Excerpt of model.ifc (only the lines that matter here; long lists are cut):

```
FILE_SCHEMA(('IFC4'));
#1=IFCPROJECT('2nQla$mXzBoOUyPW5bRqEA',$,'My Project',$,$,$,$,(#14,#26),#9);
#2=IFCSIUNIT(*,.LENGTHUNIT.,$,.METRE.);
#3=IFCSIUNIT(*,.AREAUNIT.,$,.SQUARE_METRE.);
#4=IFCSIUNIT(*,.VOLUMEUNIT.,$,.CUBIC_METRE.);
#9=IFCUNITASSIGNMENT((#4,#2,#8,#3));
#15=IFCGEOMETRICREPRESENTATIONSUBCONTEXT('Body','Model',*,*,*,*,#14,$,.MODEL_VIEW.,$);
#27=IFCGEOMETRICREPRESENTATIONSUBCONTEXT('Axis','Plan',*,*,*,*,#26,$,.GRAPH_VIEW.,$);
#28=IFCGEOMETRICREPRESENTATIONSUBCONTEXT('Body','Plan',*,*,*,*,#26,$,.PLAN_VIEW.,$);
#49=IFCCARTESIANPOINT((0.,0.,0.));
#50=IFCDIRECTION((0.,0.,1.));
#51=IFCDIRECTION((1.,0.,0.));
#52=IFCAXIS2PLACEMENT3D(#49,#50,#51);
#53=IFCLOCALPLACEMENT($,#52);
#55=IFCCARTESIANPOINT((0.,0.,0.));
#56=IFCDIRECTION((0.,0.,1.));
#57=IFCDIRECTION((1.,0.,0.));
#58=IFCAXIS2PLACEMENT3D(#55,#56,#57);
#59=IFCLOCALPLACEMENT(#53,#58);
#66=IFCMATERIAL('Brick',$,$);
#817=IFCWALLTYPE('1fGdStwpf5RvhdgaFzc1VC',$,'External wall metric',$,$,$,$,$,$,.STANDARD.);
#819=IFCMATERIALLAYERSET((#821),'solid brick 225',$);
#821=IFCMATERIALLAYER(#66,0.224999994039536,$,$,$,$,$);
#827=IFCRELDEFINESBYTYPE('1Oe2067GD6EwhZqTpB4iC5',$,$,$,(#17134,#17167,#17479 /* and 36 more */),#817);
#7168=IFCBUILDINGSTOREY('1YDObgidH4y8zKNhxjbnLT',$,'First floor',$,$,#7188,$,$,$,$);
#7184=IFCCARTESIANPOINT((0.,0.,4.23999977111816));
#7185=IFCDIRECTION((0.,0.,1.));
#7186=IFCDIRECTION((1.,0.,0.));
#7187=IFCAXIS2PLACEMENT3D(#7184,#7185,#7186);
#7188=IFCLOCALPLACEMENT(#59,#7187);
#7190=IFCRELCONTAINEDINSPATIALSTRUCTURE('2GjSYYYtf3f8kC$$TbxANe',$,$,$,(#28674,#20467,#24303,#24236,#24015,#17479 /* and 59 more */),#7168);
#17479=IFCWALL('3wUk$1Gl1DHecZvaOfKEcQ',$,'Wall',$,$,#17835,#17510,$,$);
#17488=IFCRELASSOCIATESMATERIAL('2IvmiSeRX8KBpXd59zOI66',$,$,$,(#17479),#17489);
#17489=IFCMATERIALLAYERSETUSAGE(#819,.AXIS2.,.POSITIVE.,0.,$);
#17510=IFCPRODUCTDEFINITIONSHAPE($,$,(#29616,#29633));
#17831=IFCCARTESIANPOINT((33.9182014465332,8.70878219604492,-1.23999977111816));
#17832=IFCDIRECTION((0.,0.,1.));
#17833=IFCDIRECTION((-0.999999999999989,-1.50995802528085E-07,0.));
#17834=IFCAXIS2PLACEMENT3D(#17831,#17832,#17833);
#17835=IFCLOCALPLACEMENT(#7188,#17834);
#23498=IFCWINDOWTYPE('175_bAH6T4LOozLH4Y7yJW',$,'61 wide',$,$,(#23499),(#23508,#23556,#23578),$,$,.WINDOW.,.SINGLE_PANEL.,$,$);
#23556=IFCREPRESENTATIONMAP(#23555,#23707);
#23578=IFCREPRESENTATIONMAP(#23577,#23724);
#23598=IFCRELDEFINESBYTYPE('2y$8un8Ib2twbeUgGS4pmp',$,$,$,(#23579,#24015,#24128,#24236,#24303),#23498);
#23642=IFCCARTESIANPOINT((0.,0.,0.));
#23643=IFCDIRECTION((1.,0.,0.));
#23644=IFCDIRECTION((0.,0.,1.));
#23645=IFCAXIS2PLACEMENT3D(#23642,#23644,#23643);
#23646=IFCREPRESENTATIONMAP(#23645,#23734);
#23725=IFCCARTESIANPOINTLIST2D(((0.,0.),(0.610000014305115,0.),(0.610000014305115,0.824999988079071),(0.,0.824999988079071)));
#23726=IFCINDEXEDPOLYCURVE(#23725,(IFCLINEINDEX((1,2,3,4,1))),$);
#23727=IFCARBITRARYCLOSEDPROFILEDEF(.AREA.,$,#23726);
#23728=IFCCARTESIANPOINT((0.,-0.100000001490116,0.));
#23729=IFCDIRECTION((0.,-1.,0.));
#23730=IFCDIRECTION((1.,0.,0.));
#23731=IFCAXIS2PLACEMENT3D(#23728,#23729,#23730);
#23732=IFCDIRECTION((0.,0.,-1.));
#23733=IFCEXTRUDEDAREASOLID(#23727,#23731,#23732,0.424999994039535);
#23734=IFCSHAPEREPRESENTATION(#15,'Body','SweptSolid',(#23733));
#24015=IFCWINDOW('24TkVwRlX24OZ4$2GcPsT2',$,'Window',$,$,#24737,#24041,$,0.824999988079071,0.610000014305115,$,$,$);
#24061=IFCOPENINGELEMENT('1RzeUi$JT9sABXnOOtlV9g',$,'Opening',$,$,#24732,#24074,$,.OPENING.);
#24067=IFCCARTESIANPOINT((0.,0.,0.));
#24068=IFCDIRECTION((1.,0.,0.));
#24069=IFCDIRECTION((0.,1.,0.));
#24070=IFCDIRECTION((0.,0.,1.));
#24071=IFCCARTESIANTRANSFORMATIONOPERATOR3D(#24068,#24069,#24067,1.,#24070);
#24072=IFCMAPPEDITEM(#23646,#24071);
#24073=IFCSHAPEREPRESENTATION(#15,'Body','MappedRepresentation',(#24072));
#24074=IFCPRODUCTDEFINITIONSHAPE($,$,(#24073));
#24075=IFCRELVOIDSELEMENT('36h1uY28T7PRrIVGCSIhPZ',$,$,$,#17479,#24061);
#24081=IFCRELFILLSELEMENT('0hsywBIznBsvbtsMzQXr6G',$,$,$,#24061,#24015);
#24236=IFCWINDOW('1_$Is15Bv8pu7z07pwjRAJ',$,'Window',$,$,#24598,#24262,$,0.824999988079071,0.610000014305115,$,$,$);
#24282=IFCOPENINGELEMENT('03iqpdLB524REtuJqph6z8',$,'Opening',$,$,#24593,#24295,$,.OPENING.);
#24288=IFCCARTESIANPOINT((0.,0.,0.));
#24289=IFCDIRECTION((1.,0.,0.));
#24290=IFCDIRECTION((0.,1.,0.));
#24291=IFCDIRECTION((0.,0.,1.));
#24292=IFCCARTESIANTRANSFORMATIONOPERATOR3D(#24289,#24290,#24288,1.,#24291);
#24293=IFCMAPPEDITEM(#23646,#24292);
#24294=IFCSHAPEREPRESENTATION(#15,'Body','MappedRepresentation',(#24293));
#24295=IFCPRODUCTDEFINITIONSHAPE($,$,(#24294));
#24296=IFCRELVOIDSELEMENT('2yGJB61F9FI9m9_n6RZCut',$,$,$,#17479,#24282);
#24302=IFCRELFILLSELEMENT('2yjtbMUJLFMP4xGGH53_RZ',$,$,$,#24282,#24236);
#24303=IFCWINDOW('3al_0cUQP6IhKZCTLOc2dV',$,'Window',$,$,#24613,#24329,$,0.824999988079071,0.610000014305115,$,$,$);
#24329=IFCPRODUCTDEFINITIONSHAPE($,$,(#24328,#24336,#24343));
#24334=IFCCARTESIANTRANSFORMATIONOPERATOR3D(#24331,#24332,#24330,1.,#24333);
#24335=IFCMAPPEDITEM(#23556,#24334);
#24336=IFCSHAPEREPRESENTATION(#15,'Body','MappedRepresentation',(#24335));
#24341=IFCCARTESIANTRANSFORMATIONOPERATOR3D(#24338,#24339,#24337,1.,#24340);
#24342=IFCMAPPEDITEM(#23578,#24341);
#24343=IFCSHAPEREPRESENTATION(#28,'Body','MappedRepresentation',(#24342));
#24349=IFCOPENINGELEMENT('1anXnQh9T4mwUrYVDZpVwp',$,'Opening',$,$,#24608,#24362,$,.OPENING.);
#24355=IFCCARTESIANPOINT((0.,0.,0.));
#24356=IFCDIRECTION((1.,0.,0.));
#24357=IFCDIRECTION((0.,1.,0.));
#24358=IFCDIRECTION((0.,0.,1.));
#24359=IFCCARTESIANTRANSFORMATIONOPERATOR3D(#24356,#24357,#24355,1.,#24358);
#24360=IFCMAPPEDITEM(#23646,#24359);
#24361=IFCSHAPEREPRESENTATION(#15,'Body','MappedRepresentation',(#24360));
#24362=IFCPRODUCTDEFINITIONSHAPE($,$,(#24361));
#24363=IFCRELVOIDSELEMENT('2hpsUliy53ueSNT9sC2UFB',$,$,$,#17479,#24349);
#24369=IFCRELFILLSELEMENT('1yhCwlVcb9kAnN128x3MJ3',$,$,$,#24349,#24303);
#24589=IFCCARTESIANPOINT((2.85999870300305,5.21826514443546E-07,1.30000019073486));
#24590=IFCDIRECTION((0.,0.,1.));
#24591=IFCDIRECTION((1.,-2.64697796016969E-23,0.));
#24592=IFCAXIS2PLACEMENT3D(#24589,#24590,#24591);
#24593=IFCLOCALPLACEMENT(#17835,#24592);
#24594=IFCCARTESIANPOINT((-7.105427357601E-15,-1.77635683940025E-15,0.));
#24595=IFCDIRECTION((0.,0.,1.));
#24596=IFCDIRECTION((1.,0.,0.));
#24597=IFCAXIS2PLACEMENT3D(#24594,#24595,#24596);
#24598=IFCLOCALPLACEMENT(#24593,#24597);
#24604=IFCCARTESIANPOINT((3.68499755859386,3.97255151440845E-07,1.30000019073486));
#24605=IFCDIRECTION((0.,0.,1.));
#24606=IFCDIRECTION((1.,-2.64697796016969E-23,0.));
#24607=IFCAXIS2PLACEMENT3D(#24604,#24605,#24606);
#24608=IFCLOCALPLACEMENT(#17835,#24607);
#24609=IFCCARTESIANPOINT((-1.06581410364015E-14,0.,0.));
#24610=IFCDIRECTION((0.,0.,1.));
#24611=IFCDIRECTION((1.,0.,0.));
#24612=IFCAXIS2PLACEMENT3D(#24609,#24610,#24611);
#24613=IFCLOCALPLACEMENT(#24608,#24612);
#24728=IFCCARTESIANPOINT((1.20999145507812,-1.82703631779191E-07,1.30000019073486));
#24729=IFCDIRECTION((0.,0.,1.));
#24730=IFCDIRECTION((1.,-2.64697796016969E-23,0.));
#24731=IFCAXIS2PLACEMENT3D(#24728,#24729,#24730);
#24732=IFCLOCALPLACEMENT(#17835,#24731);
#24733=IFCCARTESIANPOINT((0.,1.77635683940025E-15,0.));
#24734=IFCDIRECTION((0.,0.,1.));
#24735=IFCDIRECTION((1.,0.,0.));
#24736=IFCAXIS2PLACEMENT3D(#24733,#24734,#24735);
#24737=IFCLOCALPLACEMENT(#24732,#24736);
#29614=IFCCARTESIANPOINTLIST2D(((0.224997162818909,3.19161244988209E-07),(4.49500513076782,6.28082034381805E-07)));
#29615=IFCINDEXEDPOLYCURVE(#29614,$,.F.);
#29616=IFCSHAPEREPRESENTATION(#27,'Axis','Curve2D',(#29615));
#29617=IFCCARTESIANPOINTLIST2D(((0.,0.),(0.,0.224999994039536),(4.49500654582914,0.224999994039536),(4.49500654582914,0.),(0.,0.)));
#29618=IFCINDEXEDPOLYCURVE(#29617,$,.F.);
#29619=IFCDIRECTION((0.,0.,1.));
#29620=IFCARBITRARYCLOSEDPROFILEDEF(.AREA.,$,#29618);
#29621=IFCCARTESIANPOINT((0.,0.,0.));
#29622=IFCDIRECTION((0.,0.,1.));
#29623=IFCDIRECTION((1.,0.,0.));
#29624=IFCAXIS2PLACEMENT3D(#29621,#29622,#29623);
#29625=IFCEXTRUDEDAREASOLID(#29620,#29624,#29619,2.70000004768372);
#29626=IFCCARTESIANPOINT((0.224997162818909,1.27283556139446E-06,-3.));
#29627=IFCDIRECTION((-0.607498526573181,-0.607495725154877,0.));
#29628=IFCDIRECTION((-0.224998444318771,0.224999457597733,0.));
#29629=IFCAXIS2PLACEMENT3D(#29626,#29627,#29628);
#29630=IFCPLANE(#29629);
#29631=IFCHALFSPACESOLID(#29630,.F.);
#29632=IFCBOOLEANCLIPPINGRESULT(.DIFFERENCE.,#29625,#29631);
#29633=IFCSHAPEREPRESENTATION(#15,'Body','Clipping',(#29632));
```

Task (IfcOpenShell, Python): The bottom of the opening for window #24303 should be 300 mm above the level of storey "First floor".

```python
import numpy as np
import ifcopenshell
import ifcopenshell.api.geometry
import ifcopenshell.geom
import ifcopenshell.util.element
import ifcopenshell.util.placement
import ifcopenshell.util.shape
import ifcopenshell.util.unit

model = ifcopenshell.open("model.ifc")
unit_scale = ifcopenshell.util.unit.calculate_unit_scale(model)

window = model.by_guid("3al_0cUQP6IhKZCTLOc2dV")
opening = window.FillsVoids[0].RelatingOpeningElement
storey = ifcopenshell.util.element.get_container(window, ifc_class="IfcBuildingStorey")
level = ifcopenshell.util.placement.get_local_placement(storey.ObjectPlacement)[2, 3]

# The opening's origin need not be at the sill, so measure its lowest point.
shape = ifcopenshell.geom.create_shape(ifcopenshell.geom.settings(), opening)
bottom = ifcopenshell.util.shape.get_shape_bottom_elevation(shape, shape.geometry) / unit_scale
dz = level + 0.3 / unit_scale - bottom

shift = np.array([0.0, 0.0, dz])
# The window is placed relative to its opening, so it follows when the opening moves.
matrix = ifcopenshell.util.placement.get_local_placement(opening.ObjectPlacement)
matrix[:3, 3] += shift
ifcopenshell.api.geometry.edit_object_placement(
    model, product=opening, matrix=matrix, is_si=False, should_transform_children=True
)

print(f"moved by {dz * unit_scale:+.3f} m")

model.write("model_edited.ifc")
```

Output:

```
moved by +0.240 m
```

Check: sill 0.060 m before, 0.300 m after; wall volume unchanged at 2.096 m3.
